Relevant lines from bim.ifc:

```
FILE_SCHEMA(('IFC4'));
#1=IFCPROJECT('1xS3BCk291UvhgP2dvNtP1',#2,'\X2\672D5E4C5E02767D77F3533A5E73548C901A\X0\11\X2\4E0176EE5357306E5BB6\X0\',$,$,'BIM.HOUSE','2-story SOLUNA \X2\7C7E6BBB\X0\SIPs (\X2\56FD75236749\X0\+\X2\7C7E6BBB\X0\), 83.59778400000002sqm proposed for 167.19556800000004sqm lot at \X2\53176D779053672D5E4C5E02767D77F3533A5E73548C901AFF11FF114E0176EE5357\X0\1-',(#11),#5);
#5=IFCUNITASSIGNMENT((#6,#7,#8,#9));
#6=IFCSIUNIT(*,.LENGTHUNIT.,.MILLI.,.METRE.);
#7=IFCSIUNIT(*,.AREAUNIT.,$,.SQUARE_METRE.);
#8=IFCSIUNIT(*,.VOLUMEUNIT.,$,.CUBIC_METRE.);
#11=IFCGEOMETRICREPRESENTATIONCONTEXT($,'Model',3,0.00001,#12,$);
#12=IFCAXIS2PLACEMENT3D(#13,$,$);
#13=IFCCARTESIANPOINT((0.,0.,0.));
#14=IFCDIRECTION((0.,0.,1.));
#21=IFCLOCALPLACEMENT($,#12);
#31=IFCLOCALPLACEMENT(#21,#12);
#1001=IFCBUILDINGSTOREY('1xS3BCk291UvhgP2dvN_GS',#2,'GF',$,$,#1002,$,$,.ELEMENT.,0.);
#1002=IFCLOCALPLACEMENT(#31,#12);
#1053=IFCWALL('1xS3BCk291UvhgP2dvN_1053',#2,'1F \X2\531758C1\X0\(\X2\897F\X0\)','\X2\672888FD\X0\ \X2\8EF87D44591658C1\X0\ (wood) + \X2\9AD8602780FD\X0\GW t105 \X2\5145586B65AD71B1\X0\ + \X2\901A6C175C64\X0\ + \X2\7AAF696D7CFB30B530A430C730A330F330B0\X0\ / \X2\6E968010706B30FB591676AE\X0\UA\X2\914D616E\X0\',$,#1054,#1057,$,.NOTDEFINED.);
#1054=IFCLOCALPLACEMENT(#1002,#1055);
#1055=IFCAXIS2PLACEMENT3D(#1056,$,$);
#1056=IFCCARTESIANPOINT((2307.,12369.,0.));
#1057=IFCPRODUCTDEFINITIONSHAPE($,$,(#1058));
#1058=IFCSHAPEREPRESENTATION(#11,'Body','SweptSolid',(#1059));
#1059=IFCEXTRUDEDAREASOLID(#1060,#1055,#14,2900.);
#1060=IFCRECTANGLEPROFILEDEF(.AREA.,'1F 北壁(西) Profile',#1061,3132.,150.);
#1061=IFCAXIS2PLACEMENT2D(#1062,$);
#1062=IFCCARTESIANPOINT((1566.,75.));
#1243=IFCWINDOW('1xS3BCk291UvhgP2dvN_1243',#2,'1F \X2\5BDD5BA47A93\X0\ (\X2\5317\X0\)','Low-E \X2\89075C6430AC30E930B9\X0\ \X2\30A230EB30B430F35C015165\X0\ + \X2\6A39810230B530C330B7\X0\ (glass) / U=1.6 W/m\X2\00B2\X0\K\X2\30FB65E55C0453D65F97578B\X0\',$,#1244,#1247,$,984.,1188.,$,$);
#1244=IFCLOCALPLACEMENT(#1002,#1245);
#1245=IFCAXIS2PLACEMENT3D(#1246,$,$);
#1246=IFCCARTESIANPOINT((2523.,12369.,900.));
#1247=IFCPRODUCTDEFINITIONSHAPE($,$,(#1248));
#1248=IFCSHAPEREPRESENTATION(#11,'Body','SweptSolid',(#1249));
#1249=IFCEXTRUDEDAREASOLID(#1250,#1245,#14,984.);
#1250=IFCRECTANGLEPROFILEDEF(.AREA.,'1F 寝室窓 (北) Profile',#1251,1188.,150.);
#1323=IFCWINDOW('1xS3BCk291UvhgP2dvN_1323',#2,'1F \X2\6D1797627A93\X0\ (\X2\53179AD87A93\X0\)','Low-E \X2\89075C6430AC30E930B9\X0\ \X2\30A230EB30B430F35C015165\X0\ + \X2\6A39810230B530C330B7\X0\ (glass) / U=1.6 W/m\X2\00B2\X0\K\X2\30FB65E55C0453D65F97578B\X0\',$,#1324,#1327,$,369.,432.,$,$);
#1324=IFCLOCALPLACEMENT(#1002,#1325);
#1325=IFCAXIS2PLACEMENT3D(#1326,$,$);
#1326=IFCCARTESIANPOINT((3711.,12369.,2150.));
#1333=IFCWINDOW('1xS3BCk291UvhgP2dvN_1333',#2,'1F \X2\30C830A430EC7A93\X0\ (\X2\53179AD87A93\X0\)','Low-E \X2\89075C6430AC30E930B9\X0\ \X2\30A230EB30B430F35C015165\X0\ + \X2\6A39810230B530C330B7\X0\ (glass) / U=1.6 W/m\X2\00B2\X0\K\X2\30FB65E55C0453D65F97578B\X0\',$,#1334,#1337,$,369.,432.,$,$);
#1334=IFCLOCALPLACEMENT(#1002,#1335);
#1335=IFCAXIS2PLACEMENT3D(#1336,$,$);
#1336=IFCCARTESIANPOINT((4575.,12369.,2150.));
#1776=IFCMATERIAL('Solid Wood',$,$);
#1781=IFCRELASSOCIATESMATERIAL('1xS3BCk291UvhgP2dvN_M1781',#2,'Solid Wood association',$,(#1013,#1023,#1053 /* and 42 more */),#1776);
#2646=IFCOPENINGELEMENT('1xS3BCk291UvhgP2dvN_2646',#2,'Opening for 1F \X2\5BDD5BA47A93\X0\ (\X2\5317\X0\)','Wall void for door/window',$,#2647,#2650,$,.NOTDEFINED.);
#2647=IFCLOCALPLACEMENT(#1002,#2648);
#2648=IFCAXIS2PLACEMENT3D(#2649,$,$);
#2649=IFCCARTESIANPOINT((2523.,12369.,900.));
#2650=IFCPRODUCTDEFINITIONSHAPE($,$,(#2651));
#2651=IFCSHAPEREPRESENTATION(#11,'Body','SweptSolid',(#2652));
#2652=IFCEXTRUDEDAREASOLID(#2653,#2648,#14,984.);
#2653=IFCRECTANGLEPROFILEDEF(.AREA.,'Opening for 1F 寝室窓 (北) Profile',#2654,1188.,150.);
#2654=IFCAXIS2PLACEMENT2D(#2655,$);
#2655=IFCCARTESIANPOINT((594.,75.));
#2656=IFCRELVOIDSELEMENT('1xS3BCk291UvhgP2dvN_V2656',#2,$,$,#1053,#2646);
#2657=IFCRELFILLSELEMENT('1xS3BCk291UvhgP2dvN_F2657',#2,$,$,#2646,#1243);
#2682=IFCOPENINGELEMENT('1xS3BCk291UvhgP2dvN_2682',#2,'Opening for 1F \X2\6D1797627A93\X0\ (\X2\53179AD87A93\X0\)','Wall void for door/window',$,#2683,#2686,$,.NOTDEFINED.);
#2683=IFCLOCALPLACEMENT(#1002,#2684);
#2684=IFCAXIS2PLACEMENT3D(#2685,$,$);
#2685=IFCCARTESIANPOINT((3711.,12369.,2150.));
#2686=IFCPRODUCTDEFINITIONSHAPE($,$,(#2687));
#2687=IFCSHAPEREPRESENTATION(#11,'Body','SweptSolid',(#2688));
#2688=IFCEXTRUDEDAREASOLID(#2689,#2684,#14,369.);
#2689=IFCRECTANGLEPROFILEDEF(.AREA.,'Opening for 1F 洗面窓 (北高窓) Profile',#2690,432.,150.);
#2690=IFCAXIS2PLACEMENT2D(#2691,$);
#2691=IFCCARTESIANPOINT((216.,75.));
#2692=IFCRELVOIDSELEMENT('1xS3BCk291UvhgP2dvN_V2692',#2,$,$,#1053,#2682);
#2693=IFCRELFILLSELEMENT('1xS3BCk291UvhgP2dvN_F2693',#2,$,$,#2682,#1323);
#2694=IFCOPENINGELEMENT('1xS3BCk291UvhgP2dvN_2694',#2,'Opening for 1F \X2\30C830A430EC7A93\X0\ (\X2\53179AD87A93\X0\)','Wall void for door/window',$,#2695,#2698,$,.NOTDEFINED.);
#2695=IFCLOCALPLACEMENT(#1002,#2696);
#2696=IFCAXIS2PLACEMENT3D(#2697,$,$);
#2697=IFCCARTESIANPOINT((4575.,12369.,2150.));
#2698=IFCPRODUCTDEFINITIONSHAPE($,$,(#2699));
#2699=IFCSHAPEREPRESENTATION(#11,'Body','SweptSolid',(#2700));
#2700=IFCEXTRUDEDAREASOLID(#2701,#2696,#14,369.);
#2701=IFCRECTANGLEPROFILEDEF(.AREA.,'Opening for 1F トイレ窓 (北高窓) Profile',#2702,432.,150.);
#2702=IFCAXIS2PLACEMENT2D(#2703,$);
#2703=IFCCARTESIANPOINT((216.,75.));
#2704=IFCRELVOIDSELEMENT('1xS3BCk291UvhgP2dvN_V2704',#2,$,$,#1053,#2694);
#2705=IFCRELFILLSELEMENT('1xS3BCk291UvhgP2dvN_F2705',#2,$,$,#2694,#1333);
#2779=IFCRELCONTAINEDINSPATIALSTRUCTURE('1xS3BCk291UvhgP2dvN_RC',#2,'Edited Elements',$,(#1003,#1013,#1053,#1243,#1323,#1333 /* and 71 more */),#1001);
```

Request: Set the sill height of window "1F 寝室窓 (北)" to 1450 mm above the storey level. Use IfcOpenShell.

```python
import numpy as np
import ifcopenshell
import ifcopenshell.api.geometry
import ifcopenshell.geom
import ifcopenshell.util.element
import ifcopenshell.util.placement
import ifcopenshell.util.shape
import ifcopenshell.util.unit

model = ifcopenshell.open("bim.ifc")
unit_scale = ifcopenshell.util.unit.calculate_unit_scale(model)

window = model.by_guid("1xS3BCk291UvhgP2dvN_1243")
opening = window.FillsVoids[0].RelatingOpeningElement
storey = ifcopenshell.util.element.get_container(window, ifc_class="IfcBuildingStorey")
level = ifcopenshell.util.placement.get_local_placement(storey.ObjectPlacement)[2, 3]

# The opening's origin need not be at the sill, so measure its lowest point.
shape = ifcopenshell.geom.create_shape(ifcopenshell.geom.settings(), opening)
bottom = ifcopenshell.util.shape.get_shape_bottom_elevation(shape, shape.geometry) / unit_scale
dz = level + 1450.0 - bottom

shift = np.array([0.0, 0.0, dz])
# The window is not placed relative to its opening, so move both.
for product in (opening, window):
    matrix = ifcopenshell.util.placement.get_local_placement(product.ObjectPlacement)
    matrix[:3, 3] += shift
    ifcopenshell.api.geometry.edit_object_placement(model, product=product, matrix=matrix, is_si=False)

print(f"moved by {dz * unit_scale:+.3f} m")

model.write("bim-out.ifc")
```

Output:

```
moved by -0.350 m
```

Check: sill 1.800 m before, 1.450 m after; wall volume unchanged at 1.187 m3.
